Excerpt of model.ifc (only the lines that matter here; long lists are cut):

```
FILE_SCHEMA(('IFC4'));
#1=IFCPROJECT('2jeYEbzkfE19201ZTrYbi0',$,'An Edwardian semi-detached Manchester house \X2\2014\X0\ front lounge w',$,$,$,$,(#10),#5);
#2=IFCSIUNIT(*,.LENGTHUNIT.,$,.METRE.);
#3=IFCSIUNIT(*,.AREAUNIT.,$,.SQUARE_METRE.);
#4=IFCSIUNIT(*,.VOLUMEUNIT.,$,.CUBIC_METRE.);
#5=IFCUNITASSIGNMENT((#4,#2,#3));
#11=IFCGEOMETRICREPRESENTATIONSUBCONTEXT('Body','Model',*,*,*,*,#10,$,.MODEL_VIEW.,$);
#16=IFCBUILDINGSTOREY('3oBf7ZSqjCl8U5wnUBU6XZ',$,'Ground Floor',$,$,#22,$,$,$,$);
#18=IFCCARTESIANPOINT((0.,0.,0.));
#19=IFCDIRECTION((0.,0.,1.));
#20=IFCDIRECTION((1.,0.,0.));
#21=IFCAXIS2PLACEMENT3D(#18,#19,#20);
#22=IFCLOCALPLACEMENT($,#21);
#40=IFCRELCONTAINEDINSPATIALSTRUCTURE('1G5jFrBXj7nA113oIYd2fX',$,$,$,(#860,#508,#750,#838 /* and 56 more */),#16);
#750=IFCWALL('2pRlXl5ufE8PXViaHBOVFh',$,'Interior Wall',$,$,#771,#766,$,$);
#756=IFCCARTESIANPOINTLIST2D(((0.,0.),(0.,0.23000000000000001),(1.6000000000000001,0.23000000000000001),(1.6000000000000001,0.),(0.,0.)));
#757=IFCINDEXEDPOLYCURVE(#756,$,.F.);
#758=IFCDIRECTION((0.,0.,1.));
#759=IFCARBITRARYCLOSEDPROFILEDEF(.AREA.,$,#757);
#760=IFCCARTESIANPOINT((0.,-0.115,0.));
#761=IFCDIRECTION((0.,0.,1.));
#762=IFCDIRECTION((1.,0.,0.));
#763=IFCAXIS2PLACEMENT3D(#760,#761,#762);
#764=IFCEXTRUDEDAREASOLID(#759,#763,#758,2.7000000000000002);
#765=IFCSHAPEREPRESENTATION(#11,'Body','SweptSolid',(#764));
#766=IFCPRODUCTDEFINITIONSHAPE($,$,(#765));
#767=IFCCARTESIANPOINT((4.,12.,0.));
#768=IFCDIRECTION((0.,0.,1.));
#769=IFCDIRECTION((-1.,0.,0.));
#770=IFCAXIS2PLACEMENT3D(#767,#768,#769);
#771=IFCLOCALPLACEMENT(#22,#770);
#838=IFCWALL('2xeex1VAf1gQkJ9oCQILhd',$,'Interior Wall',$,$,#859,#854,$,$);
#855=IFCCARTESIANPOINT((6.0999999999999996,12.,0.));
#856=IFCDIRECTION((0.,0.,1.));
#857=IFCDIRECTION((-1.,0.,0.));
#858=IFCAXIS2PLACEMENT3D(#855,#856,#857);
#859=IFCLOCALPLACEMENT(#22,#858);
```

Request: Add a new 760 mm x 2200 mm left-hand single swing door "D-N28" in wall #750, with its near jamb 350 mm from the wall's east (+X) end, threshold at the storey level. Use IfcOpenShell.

```python
import numpy as np
import ifcopenshell
import ifcopenshell.api.feature
import ifcopenshell.api.geometry
import ifcopenshell.api.root
import ifcopenshell.api.spatial
import ifcopenshell.geom
import ifcopenshell.util.element
import ifcopenshell.util.placement
import ifcopenshell.util.representation
import ifcopenshell.util.shape
import ifcopenshell.util.unit

model = ifcopenshell.open("model.ifc")
unit_scale = ifcopenshell.util.unit.calculate_unit_scale(model)
settings = ifcopenshell.geom.settings()


def volume(element):
    """Net volume in cubic metres, openings subtracted."""
    shape = ifcopenshell.geom.create_shape(settings, element)
    return ifcopenshell.util.shape.get_volume(shape.geometry)


wall = model.by_guid("2pRlXl5ufE8PXViaHBOVFh")
storey = ifcopenshell.util.element.get_container(wall, ifc_class="IfcBuildingStorey")
context = ifcopenshell.util.representation.get_context(model, "Model", "Body", "MODEL_VIEW")
before = volume(wall)

width, height, from_end, sill = 0.76, 2.2, 0.35, 0.0  # metres

# The wall runs along its own X axis, and the end named is its -X end.
wall_shape = ifcopenshell.geom.create_shape(settings, wall)
x, y, z = ifcopenshell.util.shape.get_vertices(wall_shape.geometry).T
start = x.min() + from_end
face, thickness = float(y.min()), float(y.max() - y.min())
wall_matrix = ifcopenshell.util.placement.get_local_placement(wall.ObjectPlacement)
level = ifcopenshell.util.placement.get_local_placement(storey.ObjectPlacement)[2, 3]


def in_wall(x, y):
    """Placement at x, y metres in the wall's axes, at sill height."""
    matrix = wall_matrix.copy()
    matrix[:, 3] = wall_matrix @ np.array([x / unit_scale, y / unit_scale, 0.0, 1.0])
    matrix[2, 3] = level + sill / unit_scale
    return matrix


# Opening: a box that overshoots both wall faces by 50 mm.
opening = ifcopenshell.api.root.create_entity(model, ifc_class="IfcOpeningElement", predefined_type="OPENING")
box = ifcopenshell.api.geometry.add_wall_representation(
    model, context=context, length=width, height=height, thickness=thickness + 0.1
)
ifcopenshell.api.geometry.assign_representation(model, product=opening, representation=box)
ifcopenshell.api.geometry.edit_object_placement(model, product=opening, matrix=in_wall(start, face - 0.05), is_si=False)
ifcopenshell.api.feature.add_feature(model, feature=opening, element=wall)

door = ifcopenshell.api.root.create_entity(model, ifc_class="IfcDoor", name="D-N28", predefined_type="DOOR")
door.OverallWidth, door.OverallHeight = width / unit_scale, height / unit_scale
door.OperationType = "SINGLE_SWING_LEFT"
body = ifcopenshell.api.geometry.add_door_representation(
    model,
    context=context,
    overall_width=door.OverallWidth,
    overall_height=door.OverallHeight,
    operation_type="SINGLE_SWING_LEFT",
    lining_properties={"LiningDepth": thickness / unit_scale, "ThresholdDepth": thickness / unit_scale},
)
ifcopenshell.api.geometry.assign_representation(model, product=door, representation=body)
ifcopenshell.api.spatial.assign_container(model, products=[door], relating_structure=storey)
ifcopenshell.api.feature.add_filling(model, opening=opening, element=door)

# The lining spans the wall, so the door starts at the wall face.
ifcopenshell.api.geometry.edit_object_placement(model, product=door, matrix=in_wall(start, face), is_si=False)

after = volume(wall)

print(f"wall volume {before:.3f} -> {after:.3f} m3")

model.write("model-out.ifc")
```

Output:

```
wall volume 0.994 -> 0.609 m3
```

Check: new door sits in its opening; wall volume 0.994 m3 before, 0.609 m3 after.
